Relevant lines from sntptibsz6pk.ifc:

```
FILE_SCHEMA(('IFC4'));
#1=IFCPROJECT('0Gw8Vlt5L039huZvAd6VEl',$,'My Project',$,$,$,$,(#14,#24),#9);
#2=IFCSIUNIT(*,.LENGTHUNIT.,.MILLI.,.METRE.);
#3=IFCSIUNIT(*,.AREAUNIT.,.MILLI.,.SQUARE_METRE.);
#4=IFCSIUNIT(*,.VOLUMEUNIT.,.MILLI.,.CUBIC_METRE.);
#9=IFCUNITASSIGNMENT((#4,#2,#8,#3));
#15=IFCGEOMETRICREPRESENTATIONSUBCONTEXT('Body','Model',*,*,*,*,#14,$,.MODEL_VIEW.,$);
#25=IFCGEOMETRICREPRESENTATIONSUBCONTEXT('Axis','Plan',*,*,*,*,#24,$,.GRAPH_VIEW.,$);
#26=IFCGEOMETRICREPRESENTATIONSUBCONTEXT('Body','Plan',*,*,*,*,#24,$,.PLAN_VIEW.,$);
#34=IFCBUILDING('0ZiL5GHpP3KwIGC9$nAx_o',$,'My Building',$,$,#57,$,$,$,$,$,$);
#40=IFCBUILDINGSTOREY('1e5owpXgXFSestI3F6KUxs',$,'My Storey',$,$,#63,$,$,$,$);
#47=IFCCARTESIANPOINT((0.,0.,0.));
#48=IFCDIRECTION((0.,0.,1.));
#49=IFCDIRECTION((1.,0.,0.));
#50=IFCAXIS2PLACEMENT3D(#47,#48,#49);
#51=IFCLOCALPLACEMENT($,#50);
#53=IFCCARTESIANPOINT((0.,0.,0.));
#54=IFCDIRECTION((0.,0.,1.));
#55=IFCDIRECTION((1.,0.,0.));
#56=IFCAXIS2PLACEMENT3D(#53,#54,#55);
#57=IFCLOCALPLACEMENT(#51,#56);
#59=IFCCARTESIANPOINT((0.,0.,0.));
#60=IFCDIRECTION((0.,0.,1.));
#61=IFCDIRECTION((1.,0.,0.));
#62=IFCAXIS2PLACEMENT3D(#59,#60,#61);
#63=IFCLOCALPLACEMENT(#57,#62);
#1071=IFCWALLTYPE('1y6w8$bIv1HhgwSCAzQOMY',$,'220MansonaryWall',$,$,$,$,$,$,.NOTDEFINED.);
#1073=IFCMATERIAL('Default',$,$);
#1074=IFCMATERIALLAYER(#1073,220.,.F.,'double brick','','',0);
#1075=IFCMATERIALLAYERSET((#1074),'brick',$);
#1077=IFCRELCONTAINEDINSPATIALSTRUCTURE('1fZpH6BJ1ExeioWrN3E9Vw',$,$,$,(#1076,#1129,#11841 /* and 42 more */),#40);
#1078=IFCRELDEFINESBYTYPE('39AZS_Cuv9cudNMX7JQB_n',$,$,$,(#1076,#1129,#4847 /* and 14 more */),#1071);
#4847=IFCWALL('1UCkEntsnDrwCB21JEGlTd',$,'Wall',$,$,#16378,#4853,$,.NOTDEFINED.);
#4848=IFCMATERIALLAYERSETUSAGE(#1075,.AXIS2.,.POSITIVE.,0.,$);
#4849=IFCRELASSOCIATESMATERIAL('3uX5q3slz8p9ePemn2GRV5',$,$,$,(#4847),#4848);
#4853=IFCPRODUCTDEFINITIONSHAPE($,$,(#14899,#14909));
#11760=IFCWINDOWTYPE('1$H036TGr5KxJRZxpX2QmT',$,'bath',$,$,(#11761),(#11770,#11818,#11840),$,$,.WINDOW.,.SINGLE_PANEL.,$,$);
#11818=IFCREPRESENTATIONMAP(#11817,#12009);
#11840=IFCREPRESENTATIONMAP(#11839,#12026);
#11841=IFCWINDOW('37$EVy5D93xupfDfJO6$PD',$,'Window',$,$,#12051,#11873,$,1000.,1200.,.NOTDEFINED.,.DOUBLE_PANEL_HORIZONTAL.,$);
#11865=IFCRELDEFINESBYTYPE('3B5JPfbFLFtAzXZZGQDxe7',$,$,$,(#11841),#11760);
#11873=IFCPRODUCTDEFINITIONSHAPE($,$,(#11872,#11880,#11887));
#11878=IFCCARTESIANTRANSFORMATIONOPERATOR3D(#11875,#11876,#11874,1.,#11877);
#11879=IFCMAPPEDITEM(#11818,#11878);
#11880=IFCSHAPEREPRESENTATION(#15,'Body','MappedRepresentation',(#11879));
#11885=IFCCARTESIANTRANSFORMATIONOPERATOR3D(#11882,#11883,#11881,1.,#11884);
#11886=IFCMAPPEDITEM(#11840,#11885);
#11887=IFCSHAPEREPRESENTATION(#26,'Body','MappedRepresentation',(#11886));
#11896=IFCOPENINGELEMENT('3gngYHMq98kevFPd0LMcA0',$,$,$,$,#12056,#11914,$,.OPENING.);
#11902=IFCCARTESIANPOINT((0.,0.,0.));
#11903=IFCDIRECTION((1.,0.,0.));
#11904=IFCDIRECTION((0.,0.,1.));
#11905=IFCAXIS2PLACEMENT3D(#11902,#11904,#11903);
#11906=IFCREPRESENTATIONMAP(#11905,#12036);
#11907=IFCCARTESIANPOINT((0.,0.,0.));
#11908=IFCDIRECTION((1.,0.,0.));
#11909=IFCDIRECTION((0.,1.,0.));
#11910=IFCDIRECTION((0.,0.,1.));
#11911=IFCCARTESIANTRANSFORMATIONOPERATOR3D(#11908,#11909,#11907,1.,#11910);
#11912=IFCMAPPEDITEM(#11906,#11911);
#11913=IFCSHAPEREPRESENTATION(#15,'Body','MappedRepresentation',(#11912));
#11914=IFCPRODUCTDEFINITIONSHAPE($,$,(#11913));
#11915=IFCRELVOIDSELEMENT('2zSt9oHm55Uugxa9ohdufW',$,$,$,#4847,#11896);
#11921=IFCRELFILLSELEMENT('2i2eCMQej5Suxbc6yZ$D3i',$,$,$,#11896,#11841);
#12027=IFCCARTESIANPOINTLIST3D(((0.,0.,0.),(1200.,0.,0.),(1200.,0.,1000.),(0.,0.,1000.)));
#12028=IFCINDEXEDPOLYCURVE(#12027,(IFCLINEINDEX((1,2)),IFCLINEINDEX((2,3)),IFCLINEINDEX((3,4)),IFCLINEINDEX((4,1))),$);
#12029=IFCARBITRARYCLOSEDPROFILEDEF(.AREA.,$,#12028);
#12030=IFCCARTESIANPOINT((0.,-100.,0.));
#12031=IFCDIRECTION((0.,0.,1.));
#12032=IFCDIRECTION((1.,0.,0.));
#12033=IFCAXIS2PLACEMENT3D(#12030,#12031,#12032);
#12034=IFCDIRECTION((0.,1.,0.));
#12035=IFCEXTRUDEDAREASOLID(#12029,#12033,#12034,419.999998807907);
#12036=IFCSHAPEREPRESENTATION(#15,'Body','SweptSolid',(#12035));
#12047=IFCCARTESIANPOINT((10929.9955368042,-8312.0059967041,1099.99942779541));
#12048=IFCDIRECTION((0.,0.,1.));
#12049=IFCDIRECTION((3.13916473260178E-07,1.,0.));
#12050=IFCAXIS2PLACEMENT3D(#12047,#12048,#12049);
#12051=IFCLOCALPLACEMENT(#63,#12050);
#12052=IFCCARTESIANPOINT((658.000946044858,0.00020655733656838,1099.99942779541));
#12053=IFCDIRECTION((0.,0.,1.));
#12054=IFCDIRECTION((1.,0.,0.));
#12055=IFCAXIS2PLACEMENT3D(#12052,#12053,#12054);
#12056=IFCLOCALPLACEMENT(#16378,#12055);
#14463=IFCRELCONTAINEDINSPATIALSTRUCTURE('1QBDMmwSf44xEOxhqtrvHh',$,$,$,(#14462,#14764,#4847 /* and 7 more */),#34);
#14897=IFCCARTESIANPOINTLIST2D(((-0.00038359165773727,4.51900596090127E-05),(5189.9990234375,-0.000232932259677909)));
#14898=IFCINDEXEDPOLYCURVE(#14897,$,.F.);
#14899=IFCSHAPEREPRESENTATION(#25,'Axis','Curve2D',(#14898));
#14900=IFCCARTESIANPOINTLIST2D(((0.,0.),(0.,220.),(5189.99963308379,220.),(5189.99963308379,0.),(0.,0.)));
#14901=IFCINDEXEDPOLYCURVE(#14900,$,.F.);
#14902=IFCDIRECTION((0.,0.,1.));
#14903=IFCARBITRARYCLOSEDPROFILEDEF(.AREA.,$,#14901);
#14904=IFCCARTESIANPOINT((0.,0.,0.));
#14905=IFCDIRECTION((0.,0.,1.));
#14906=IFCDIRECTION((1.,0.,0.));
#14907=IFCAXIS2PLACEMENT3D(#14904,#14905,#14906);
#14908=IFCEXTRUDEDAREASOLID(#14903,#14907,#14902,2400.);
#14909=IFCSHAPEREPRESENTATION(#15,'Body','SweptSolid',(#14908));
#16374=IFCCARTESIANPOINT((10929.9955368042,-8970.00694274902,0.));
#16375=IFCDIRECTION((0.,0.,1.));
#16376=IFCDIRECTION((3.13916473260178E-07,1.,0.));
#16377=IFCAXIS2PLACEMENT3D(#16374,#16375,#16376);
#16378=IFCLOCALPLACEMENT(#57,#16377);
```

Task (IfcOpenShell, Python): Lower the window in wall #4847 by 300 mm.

```python
import numpy as np
import ifcopenshell
import ifcopenshell.api.geometry
import ifcopenshell.util.placement
import ifcopenshell.util.unit

model = ifcopenshell.open("sntptibsz6pk.ifc")
unit_scale = ifcopenshell.util.unit.calculate_unit_scale(model)

window = model.by_id(11841)
opening = window.FillsVoids[0].RelatingOpeningElement
dz = -300.0

shift = np.array([0.0, 0.0, dz])
# The window is not placed relative to its opening, so move both.
for product in (opening, window):
    matrix = ifcopenshell.util.placement.get_local_placement(product.ObjectPlacement)
    matrix[:3, 3] += shift
    ifcopenshell.api.geometry.edit_object_placement(model, product=product, matrix=matrix, is_si=False)

print(f"moved by {dz * unit_scale:+.3f} m")

model.write("sntptibsz6pk_rev.ifc")
```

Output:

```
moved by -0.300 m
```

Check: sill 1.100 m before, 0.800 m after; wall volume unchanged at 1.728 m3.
